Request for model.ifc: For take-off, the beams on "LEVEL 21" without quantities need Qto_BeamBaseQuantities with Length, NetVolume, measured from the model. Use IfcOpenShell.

First a look at what the model holds.

```python
import ifcopenshell
import ifcopenshell.util.element
import ifcopenshell.util.unit

model = ifcopenshell.open("model.ifc")
print(model.schema)
for unit_type in ("LENGTHUNIT", "AREAUNIT", "VOLUMEUNIT"):
    print(unit_type, ifcopenshell.util.unit.calculate_unit_scale(model, unit_type))
storey = next(s for s in model.by_type("IfcBuildingStorey") if s.Name == "LEVEL 21")
beams = [e for e in ifcopenshell.util.element.get_decomposition(storey) if e.is_a("IfcBeam")]
for e in sorted(beams, key=lambda e: e.id()):
    print(e.id(), e.is_a(), e.Name, list(ifcopenshell.util.element.get_psets(e, qtos_only=True)), sep=" | ")
```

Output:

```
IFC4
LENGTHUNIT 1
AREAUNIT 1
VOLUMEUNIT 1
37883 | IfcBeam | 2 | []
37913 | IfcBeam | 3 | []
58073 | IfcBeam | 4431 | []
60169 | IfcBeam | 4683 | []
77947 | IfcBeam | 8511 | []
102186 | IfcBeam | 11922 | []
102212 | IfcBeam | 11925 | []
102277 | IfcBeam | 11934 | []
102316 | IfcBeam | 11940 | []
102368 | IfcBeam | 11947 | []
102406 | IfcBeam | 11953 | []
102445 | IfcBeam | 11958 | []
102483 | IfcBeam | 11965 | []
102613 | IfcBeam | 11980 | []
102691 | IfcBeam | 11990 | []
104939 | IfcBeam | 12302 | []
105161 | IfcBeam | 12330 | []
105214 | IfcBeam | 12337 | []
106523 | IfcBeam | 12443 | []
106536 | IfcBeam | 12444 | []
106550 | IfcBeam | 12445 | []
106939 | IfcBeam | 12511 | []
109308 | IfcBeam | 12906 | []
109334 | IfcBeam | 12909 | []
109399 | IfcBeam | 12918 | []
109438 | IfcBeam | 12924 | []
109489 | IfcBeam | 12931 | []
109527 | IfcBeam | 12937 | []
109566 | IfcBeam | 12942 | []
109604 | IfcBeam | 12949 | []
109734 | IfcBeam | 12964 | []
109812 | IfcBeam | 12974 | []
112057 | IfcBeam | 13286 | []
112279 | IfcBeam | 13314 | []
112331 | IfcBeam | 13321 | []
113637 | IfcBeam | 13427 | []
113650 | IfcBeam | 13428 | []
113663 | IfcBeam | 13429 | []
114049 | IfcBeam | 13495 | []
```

```python
import ifcopenshell
import ifcopenshell.api.pset
import ifcopenshell.geom
import ifcopenshell.util.element
import ifcopenshell.util.shape
import ifcopenshell.util.unit

model = ifcopenshell.open("model.ifc")
unit_scale = ifcopenshell.util.unit.calculate_unit_scale(model)
volume_scale = ifcopenshell.util.unit.calculate_unit_scale(model, "VOLUMEUNIT")
settings = ifcopenshell.geom.settings()

storey = next(s for s in model.by_type("IfcBuildingStorey") if s.Name == "LEVEL 21")
beams = [e for e in ifcopenshell.util.element.get_decomposition(storey) if e.is_a("IfcBeam")]

for e in sorted(beams, key=lambda e: e.id()):
    if ifcopenshell.util.element.get_psets(e, qtos_only=True, should_inherit=False):
        continue
    # Geometry comes back in metres, in the element's own axes.
    shape = ifcopenshell.geom.create_shape(settings, e)
    values = {
        "Length": ifcopenshell.util.shape.get_max_xyz(shape.geometry) / unit_scale,
        "NetVolume": ifcopenshell.util.shape.get_volume(shape.geometry) / volume_scale,
    }
    qto = ifcopenshell.api.pset.add_qto(model, product=e, name="Qto_BeamBaseQuantities")
    ifcopenshell.api.pset.edit_qto(model, qto=qto, properties=values)
    print(e.id(), {k: round(v, 3) for k, v in values.items()})

model.write("model-out.ifc")
```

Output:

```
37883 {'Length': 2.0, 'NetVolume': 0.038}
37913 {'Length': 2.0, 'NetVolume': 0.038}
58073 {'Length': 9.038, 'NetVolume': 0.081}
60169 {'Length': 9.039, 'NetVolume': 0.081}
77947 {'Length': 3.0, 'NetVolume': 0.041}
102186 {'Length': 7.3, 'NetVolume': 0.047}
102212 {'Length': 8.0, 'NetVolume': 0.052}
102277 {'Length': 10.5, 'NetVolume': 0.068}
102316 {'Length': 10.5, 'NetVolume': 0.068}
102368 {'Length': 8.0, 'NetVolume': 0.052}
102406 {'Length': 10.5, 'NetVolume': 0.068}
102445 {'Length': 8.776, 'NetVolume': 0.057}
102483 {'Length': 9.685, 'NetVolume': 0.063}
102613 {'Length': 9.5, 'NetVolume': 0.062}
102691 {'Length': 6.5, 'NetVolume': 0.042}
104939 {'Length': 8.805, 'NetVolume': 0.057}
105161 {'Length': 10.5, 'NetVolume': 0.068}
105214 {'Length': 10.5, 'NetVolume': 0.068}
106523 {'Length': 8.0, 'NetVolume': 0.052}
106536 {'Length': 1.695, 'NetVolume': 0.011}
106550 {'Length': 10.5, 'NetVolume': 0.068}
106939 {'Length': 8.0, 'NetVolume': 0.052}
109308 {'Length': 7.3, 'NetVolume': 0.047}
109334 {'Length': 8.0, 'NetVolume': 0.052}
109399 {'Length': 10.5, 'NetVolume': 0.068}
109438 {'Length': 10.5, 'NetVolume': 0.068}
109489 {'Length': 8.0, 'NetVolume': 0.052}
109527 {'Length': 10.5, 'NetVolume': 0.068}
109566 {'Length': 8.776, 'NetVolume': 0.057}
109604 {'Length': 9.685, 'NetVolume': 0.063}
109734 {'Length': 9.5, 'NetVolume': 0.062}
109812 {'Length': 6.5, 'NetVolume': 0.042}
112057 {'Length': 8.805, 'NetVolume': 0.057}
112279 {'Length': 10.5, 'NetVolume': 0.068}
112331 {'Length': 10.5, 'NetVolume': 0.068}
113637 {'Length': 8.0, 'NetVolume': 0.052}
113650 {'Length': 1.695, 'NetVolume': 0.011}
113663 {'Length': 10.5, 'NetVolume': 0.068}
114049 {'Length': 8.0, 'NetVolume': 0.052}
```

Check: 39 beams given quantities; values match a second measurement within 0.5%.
